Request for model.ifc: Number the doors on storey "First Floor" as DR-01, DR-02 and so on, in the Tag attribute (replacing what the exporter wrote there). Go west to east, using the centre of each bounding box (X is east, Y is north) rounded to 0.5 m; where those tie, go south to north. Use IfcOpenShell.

First a look at what the model holds.

```python
import ifcopenshell
import ifcopenshell.util.element
import ifcopenshell.util.placement

model = ifcopenshell.open("model.ifc")
print(model.schema)
storey = next(s for s in model.by_type("IfcBuildingStorey") if s.Name == "First Floor")
doors = [e for e in ifcopenshell.util.element.get_decomposition(storey) if e.is_a("IfcDoor")]
for e in sorted(doors, key=lambda e: e.id()):
    origin = ifcopenshell.util.placement.get_local_placement(e.ObjectPlacement)[:3, 3]
    print(e.id(), e.Tag, e.Name, origin.round(2) + 0.0, sep=" | ")
```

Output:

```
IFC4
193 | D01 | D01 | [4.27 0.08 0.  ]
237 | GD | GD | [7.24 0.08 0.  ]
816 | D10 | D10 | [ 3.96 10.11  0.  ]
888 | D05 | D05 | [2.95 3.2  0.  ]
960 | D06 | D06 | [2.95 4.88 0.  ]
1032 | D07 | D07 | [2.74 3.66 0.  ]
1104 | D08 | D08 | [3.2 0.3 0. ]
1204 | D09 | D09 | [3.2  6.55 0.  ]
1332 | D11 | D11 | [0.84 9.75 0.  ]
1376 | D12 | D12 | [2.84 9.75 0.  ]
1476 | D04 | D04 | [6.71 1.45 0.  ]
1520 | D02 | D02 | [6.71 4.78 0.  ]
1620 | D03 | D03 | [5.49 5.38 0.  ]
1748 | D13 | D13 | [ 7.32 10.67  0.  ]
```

```python
import ifcopenshell
import ifcopenshell.geom
import ifcopenshell.util.element
import ifcopenshell.util.shape

model = ifcopenshell.open("model.ifc")
settings = ifcopenshell.geom.settings()
settings.set("use-world-coords", True)


def centre(element):
    shape = ifcopenshell.geom.create_shape(settings, element)
    return ifcopenshell.util.shape.get_bbox_centroid(shape.geometry)


storey = next(s for s in model.by_type("IfcBuildingStorey") if s.Name == "First Floor")
doors = [e for e in ifcopenshell.util.element.get_decomposition(storey) if e.is_a("IfcDoor")]

# Insertion points can sit at a corner or the storey origin, so sort by the geometry (in metres).
centres = {e: centre(e) for e in doors}
doors.sort(key=lambda e: (round(centres[e][0] / 0.5), centres[e][1]))

for i, e in enumerate(doors, start=1):
    number = f"DR-{i:02d}"
    e.Tag = number
    print(e.id(), number)

model.write("model-out.ifc")
```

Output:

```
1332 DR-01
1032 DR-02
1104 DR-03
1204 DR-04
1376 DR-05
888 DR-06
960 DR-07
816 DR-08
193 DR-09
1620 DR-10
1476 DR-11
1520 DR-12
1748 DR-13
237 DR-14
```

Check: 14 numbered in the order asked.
